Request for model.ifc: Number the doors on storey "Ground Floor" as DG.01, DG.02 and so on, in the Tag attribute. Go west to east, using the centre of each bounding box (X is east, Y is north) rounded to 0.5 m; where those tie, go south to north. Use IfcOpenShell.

First a look at what the model holds.

```python
import ifcopenshell
import ifcopenshell.util.element
import ifcopenshell.util.placement

model = ifcopenshell.open("model.ifc")
print(model.schema)
storey = next(s for s in model.by_type("IfcBuildingStorey") if s.Name == "Ground Floor")
doors = [e for e in ifcopenshell.util.element.get_decomposition(storey) if e.is_a("IfcDoor")]
for e in sorted(doors, key=lambda e: e.id()):
    origin = ifcopenshell.util.placement.get_local_placement(e.ObjectPlacement)[:3, 3]
    print(e.id(), e.Tag, e.Name, origin.round(2) + 0.0, sep=" | ")
```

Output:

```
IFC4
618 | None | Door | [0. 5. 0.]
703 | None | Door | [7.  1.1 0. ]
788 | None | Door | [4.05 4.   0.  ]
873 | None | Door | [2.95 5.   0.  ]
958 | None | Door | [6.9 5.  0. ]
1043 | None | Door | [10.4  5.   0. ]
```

```python
import ifcopenshell
import ifcopenshell.geom
import ifcopenshell.util.element
import ifcopenshell.util.shape

model = ifcopenshell.open("model.ifc")
settings = ifcopenshell.geom.settings()
settings.set("use-world-coords", True)


def centre(element):
    shape = ifcopenshell.geom.create_shape(settings, element)
    return ifcopenshell.util.shape.get_bbox_centroid(shape.geometry)


storey = next(s for s in model.by_type("IfcBuildingStorey") if s.Name == "Ground Floor")
doors = [e for e in ifcopenshell.util.element.get_decomposition(storey) if e.is_a("IfcDoor")]

# Insertion points can sit at a corner or the storey origin, so sort by the geometry (in metres).
centres = {e: centre(e) for e in doors}
doors.sort(key=lambda e: (round(centres[e][0] / 0.5), centres[e][1]))

for i, e in enumerate(doors, start=1):
    number = f"DG.{i:02d}"
    e.Tag = number
    print(e.id(), number)

model.write("model_updated.ifc")
```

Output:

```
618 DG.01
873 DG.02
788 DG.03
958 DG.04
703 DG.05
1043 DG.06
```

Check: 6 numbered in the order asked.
